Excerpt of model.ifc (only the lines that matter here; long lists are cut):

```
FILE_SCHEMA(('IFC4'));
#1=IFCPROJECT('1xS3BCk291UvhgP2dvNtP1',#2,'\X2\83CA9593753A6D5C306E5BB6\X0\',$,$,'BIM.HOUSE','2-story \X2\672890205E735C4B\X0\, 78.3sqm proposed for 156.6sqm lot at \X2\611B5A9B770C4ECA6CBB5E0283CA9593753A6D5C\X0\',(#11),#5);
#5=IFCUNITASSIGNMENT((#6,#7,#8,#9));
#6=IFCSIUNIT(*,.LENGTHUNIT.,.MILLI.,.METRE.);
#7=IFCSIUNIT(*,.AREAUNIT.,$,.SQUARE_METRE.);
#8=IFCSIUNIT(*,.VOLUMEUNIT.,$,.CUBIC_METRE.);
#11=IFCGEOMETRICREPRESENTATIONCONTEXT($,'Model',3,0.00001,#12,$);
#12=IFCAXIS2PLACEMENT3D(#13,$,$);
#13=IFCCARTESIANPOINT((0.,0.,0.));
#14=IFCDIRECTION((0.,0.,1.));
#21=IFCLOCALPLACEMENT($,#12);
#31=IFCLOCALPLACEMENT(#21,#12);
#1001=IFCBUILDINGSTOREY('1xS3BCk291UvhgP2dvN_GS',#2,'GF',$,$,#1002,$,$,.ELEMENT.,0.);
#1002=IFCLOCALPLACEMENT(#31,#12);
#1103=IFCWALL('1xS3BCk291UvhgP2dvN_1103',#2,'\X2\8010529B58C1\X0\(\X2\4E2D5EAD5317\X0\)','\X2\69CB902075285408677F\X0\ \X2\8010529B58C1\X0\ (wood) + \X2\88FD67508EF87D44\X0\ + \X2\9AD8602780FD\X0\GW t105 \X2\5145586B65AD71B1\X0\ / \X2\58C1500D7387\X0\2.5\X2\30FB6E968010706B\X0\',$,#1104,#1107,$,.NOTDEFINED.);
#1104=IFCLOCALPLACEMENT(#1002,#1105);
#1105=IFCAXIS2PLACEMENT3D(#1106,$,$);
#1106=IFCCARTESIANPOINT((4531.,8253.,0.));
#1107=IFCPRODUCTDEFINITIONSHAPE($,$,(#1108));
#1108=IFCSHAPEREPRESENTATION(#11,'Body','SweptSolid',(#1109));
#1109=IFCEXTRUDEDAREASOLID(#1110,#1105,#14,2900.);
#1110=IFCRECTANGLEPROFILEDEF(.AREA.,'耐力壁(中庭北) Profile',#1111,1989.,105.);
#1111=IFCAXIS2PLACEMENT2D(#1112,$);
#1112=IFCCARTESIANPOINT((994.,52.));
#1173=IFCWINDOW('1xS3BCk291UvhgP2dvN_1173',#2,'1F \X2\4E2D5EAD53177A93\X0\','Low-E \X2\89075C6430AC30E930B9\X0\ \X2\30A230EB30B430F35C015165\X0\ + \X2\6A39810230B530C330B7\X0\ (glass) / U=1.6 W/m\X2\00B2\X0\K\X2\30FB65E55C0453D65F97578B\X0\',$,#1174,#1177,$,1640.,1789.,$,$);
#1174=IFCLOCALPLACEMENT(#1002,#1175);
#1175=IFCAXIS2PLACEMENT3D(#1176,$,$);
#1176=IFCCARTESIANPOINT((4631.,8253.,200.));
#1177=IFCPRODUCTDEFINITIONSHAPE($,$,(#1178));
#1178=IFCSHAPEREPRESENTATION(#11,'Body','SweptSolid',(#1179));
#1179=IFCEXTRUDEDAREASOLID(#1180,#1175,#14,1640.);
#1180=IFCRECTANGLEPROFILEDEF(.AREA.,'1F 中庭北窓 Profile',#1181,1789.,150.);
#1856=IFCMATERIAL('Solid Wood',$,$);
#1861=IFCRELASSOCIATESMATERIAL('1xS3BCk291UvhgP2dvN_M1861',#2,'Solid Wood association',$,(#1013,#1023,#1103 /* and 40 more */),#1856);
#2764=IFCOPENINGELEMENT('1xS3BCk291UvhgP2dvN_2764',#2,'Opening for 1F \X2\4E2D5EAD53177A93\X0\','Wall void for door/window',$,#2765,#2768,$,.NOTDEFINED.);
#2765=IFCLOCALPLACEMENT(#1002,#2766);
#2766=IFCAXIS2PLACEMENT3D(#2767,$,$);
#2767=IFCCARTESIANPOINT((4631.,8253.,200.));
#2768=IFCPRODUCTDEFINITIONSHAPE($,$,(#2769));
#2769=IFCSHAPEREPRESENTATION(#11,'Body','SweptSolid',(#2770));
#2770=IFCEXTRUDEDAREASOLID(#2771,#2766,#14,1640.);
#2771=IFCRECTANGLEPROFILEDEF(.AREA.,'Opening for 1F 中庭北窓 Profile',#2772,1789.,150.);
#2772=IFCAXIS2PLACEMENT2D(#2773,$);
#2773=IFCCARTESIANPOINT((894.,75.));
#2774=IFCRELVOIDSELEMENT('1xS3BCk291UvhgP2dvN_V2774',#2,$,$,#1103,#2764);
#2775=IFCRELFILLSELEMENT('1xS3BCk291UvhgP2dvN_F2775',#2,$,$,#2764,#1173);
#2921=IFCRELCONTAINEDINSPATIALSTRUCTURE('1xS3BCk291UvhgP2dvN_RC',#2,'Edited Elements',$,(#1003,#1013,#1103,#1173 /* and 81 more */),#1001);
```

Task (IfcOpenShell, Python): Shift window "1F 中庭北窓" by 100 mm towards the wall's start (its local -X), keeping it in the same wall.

```python
import ifcopenshell
import ifcopenshell.api.geometry
import ifcopenshell.util.placement
import ifcopenshell.util.unit

model = ifcopenshell.open("model.ifc")
unit_scale = ifcopenshell.util.unit.calculate_unit_scale(model)

window = model.by_guid("1xS3BCk291UvhgP2dvN_1173")
opening = window.FillsVoids[0].RelatingOpeningElement
wall = opening.VoidsElements[0].RelatingBuildingElement

wall_matrix = ifcopenshell.util.placement.get_local_placement(wall.ObjectPlacement)
shift = wall_matrix[:3, 0] * -0.1 / unit_scale
before = ifcopenshell.util.placement.get_local_placement(window.ObjectPlacement)[:3, 3].copy()

# The window is not placed relative to its opening, so move both.
for product in (opening, window):
    matrix = ifcopenshell.util.placement.get_local_placement(product.ObjectPlacement)
    matrix[:3, 3] += shift
    ifcopenshell.api.geometry.edit_object_placement(model, product=product, matrix=matrix, is_si=False)

after = ifcopenshell.util.placement.get_local_placement(window.ObjectPlacement)[:3, 3]
print("window moved by", (after - before).round(3) + 0.0)

model.write("model_rev.ifc")
```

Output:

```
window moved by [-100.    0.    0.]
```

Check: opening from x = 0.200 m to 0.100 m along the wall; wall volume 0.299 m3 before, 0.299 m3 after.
